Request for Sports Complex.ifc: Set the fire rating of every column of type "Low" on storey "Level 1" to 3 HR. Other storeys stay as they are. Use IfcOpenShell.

First a look at what the model holds.

```python
import ifcopenshell
import ifcopenshell.util.element

model = ifcopenshell.open("Sports Complex.ifc")
print(model.schema)
storey = next(s for s in model.by_type("IfcBuildingStorey") if s.Name == "Level 1")
columns = [e for e in ifcopenshell.util.element.get_decomposition(storey) if e.is_a("IfcColumn")]
seen = {}
for e in columns:
    element_type = ifcopenshell.util.element.get_type(e)
    key = (element_type.Name if element_type != e and element_type else None, ifcopenshell.util.element.get_pset(e, "Pset_ColumnCommon", "FireRating"))
    seen[key] = seen.get(key, 0) + 1
for (name, value), count in sorted(seen.items(), key=str):
    print(count, "x", name, "|", value)
```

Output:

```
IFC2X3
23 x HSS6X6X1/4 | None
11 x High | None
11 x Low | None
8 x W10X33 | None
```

```python
import ifcopenshell
import ifcopenshell.api.pset
import ifcopenshell.util.element

model = ifcopenshell.open("Sports Complex.ifc")

storey = next(s for s in model.by_type("IfcBuildingStorey") if s.Name == "Level 1")
columns = [e for e in ifcopenshell.util.element.get_decomposition(storey) if e.is_a("IfcColumn")]

count = 0
for e in columns:
    element_type = ifcopenshell.util.element.get_type(e)
    if element_type in (None, e) or element_type.Name != "Low":
        continue
    # add_pset returns the element's existing set when there is one.
    pset = ifcopenshell.api.pset.add_pset(model, product=e, name="Pset_ColumnCommon")
    ifcopenshell.api.pset.edit_pset(model, pset=pset, properties={"FireRating": "3 HR"})
    count += 1

print(count, "columns updated")

model.write("Sports Complex_rev.ifc")
```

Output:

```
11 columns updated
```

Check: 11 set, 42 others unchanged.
